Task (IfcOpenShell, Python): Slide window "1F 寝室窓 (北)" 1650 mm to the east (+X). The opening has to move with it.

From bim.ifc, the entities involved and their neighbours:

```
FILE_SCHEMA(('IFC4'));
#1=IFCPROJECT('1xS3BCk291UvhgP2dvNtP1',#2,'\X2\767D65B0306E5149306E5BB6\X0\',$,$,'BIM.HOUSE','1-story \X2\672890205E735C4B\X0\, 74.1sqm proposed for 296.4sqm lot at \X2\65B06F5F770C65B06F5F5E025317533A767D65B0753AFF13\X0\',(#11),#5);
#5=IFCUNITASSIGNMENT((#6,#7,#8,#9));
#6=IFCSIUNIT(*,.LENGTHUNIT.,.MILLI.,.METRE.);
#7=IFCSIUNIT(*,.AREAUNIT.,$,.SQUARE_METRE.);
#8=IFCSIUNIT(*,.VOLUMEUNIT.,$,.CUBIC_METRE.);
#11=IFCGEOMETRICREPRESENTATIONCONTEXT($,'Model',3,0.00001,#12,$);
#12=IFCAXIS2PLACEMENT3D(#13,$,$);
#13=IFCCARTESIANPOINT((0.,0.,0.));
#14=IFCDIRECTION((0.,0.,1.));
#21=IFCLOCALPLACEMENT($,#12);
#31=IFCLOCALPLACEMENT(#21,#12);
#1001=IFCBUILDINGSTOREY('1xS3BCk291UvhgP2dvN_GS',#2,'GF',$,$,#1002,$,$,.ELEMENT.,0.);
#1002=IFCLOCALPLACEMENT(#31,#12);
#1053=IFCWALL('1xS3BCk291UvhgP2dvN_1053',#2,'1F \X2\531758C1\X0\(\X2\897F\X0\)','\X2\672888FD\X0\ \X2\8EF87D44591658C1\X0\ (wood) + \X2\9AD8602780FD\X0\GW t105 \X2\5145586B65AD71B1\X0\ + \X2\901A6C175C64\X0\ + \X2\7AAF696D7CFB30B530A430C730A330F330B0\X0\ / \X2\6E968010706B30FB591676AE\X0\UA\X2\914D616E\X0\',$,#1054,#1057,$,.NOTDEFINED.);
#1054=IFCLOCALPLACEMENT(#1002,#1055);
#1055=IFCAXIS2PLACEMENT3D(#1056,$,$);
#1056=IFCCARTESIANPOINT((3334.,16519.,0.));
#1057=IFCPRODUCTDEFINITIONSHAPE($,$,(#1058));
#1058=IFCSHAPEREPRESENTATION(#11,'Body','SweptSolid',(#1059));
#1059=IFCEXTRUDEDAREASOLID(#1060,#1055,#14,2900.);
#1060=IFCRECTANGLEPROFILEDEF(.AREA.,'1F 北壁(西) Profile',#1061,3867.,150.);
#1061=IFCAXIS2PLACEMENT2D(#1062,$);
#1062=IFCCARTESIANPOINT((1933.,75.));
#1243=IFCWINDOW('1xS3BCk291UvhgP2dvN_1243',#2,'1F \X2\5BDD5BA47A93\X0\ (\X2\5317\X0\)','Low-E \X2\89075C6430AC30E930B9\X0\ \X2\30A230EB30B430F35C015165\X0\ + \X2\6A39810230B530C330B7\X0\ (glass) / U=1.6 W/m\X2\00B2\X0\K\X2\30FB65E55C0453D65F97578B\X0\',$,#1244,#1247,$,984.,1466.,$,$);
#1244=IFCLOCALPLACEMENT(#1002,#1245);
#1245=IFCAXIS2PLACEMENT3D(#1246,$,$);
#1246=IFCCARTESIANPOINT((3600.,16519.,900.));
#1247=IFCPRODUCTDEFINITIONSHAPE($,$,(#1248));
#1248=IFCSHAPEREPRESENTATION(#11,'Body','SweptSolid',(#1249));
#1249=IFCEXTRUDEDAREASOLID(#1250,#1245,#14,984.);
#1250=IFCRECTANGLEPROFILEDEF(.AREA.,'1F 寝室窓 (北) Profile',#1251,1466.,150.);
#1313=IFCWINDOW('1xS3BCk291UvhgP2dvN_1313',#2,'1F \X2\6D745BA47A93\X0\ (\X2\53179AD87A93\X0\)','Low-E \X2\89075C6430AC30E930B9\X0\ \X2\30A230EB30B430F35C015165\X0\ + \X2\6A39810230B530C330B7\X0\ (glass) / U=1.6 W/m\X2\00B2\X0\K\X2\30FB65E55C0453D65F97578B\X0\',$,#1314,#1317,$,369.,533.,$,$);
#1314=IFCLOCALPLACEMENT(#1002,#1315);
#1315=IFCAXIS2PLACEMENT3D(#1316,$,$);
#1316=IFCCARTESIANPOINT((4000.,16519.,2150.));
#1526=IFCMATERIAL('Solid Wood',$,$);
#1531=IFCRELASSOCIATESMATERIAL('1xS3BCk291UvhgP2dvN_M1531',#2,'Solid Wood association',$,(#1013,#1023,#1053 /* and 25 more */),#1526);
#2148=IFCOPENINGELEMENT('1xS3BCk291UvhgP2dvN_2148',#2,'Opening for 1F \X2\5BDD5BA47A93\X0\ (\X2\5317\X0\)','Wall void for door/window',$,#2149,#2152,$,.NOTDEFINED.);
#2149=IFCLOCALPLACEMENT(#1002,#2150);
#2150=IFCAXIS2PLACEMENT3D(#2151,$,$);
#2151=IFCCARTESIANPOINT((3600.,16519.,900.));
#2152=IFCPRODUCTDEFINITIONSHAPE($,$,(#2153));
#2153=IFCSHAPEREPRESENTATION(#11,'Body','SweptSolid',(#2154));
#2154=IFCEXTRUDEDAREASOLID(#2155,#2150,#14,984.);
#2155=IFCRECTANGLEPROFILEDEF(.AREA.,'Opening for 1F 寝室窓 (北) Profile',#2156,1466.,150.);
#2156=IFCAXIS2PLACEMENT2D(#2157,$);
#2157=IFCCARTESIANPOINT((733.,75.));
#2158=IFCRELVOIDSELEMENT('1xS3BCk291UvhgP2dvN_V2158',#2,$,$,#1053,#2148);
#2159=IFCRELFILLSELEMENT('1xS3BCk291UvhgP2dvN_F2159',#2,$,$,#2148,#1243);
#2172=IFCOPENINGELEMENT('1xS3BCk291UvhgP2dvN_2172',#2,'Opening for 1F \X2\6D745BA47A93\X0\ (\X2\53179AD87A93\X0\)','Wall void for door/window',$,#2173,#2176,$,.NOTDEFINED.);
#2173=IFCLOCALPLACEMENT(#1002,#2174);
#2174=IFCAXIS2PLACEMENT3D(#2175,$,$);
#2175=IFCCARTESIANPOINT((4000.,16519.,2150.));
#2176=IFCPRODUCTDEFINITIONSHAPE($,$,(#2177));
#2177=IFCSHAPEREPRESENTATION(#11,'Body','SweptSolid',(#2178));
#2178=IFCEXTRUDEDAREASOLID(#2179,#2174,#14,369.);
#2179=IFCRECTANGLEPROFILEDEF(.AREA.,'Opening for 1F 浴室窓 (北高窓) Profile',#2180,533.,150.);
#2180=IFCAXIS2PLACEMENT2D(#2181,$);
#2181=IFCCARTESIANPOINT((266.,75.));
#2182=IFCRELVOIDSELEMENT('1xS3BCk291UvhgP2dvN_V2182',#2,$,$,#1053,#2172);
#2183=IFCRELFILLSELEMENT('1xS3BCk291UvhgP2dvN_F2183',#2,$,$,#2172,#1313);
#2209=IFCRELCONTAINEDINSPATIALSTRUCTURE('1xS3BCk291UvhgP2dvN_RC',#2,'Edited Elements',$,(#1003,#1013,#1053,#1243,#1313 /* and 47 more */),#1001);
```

```python
import ifcopenshell
import ifcopenshell.api.geometry
import ifcopenshell.util.placement

model = ifcopenshell.open("bim.ifc")

window = model.by_guid("1xS3BCk291UvhgP2dvN_1243")
opening = window.FillsVoids[0].RelatingOpeningElement
wall = opening.VoidsElements[0].RelatingBuildingElement

wall_matrix = ifcopenshell.util.placement.get_local_placement(wall.ObjectPlacement)
shift = wall_matrix[:3, 0] * 1650.0
before = ifcopenshell.util.placement.get_local_placement(window.ObjectPlacement)[:3, 3].copy()

# The window is not placed relative to its opening, so move both.
for product in (opening, window):
    matrix = ifcopenshell.util.placement.get_local_placement(product.ObjectPlacement)
    matrix[:3, 3] += shift
    ifcopenshell.api.geometry.edit_object_placement(model, product=product, matrix=matrix, is_si=False)

after = ifcopenshell.util.placement.get_local_placement(window.ObjectPlacement)[:3, 3]
print("window moved by", (after - before).round(3) + 0.0)

model.write("bim_edited.ifc")
```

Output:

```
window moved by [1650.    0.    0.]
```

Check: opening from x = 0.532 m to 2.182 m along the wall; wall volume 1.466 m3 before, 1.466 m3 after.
